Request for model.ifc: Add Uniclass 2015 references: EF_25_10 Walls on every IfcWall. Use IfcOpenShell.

First a look at what the model holds.

```python
import ifcopenshell

model = ifcopenshell.open("model.ifc")
print(model.schema)
print("classifications:", [c.Name for c in model.by_type("IfcClassification")])
for ifc_class in ("IfcDoor", "IfcRoof", "IfcStair", "IfcWall", "IfcWindow"):
    print(ifc_class, len(model.by_type(ifc_class)))
```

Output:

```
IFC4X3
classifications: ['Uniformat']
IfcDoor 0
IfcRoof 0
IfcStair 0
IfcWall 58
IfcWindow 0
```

```python
import ifcopenshell
import ifcopenshell.api.classification

model = ifcopenshell.open("model.ifc")

system = ifcopenshell.api.classification.add_classification(model, classification="Uniclass 2015")

codes = {
    "IfcWall": ("EF_25_10", "Walls"),
}
for ifc_class, (code, name) in codes.items():
    products = model.by_type(ifc_class)
    ifcopenshell.api.classification.add_reference(
        model, products=products, classification=system, identification=code, name=name
    )
    print(code, len(products))

model.write("model-out.ifc")
```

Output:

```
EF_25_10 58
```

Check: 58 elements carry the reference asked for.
